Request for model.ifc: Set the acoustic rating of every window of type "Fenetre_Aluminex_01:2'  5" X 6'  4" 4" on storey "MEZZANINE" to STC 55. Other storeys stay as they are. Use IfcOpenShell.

First a look at what the model holds.

```python
import ifcopenshell
import ifcopenshell.util.element

model = ifcopenshell.open("model.ifc")
print(model.schema)
storey = next(s for s in model.by_type("IfcBuildingStorey") if s.Name == "MEZZANINE")
windows = [e for e in ifcopenshell.util.element.get_decomposition(storey) if e.is_a("IfcWindow")]
seen = {}
for e in windows:
    element_type = ifcopenshell.util.element.get_type(e)
    key = (element_type.Name if element_type != e and element_type else None, ifcopenshell.util.element.get_pset(e, "Pset_WindowCommon", "AcousticRating"))
    seen[key] = seen.get(key, 0) + 1
for (name, value), count in sorted(seen.items(), key=str):
    print(count, "x", name, "|", value)
```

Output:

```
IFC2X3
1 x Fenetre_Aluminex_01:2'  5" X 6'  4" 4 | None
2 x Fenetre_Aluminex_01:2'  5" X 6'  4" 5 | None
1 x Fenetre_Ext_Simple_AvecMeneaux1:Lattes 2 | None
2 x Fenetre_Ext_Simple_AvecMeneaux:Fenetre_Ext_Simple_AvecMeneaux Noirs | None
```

```python
import ifcopenshell
import ifcopenshell.api.pset
import ifcopenshell.util.element

model = ifcopenshell.open("model.ifc")

storey = next(s for s in model.by_type("IfcBuildingStorey") if s.Name == "MEZZANINE")
windows = [e for e in ifcopenshell.util.element.get_decomposition(storey) if e.is_a("IfcWindow")]

count = 0
for e in windows:
    element_type = ifcopenshell.util.element.get_type(e)
    if element_type in (None, e) or element_type.Name != 'Fenetre_Aluminex_01:2\'  5" X 6\'  4" 4':
        continue
    # add_pset returns the element's existing set when there is one.
    pset = ifcopenshell.api.pset.add_pset(model, product=e, name="Pset_WindowCommon")
    ifcopenshell.api.pset.edit_pset(model, pset=pset, properties={"AcousticRating": "STC 55"})
    count += 1

print(count, "windows updated")

model.write("model_edited.ifc")
```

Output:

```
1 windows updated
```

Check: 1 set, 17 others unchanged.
